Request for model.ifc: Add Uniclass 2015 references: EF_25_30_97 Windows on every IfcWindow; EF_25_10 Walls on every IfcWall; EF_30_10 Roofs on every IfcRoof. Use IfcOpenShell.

First a look at what the model holds.

```python
import ifcopenshell

model = ifcopenshell.open("model.ifc")
print(model.schema)
print("classifications:", [c.Name for c in model.by_type("IfcClassification")])
for ifc_class in ("IfcDoor", "IfcRoof", "IfcStair", "IfcWall", "IfcWindow"):
    print(ifc_class, len(model.by_type(ifc_class)))
```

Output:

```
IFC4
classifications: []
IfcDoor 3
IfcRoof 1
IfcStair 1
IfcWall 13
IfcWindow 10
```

```python
import ifcopenshell
import ifcopenshell.api.classification

model = ifcopenshell.open("model.ifc")

system = ifcopenshell.api.classification.add_classification(model, classification="Uniclass 2015")

codes = {
    "IfcWindow": ("EF_25_30_97", "Windows"),
    "IfcWall": ("EF_25_10", "Walls"),
    "IfcRoof": ("EF_30_10", "Roofs"),
}
for ifc_class, (code, name) in codes.items():
    products = model.by_type(ifc_class)
    ifcopenshell.api.classification.add_reference(
        model, products=products, classification=system, identification=code, name=name
    )
    print(code, len(products))

model.write("model_edited.ifc")
```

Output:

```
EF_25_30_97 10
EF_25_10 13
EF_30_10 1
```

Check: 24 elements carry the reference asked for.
